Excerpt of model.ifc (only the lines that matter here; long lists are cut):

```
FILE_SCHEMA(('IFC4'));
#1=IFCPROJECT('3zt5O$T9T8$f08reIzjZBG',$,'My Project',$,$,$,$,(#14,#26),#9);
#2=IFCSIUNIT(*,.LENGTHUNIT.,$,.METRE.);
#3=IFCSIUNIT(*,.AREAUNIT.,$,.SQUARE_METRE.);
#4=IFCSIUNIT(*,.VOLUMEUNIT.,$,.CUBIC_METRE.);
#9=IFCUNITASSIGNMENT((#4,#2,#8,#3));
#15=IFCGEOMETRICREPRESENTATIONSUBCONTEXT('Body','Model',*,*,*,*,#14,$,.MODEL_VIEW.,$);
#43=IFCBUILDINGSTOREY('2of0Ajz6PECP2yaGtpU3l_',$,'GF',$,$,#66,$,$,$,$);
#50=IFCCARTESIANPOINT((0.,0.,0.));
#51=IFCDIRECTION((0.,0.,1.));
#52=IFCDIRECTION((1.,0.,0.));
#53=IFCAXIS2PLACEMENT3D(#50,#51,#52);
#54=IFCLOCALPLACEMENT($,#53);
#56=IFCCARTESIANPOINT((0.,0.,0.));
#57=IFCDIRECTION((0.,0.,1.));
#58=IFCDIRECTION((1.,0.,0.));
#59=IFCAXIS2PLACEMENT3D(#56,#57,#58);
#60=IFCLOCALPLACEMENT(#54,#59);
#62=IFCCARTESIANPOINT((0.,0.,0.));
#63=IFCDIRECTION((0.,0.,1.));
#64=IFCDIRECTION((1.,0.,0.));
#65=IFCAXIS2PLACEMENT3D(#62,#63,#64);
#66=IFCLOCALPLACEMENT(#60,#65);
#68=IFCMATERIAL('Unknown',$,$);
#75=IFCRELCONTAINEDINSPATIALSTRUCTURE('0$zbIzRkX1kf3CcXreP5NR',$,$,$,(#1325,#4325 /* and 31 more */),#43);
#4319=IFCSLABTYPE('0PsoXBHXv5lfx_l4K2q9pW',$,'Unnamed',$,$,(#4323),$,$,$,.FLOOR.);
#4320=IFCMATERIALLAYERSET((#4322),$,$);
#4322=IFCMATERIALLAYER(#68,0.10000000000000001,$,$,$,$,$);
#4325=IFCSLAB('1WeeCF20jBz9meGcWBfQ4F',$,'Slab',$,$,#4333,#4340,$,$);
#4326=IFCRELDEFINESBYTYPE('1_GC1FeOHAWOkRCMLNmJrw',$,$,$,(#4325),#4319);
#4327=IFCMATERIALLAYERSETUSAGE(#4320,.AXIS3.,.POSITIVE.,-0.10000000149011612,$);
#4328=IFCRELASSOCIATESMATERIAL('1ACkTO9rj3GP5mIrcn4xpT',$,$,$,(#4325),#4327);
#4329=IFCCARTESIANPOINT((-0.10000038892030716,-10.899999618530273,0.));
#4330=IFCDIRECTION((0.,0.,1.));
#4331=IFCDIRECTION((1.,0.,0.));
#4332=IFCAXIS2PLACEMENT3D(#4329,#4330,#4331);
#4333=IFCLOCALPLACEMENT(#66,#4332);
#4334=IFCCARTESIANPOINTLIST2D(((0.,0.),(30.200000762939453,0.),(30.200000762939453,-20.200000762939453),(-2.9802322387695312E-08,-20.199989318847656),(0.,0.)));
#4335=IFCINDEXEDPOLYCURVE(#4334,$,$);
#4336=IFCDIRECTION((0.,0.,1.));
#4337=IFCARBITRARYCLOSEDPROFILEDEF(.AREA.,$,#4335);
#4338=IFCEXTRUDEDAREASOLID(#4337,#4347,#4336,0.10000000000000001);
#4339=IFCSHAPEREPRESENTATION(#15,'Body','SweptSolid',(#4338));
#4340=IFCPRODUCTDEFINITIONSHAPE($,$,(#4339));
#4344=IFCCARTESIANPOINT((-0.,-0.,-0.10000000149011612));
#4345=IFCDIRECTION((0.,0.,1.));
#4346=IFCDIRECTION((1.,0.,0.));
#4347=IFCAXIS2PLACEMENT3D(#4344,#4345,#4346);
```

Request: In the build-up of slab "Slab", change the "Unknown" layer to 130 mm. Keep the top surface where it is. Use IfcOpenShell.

```python
import ifcopenshell
import ifcopenshell.util.element
import ifcopenshell.util.representation
import ifcopenshell.util.unit

model = ifcopenshell.open("model.ifc")
unit_scale = ifcopenshell.util.unit.calculate_unit_scale(model)

layer_set = model.by_id(4320)
layer = next(l for l in layer_set.MaterialLayers if l.Material and l.Material.Name == "Unknown")
change = 0.13 / unit_scale - layer.LayerThickness
layer.LayerThickness += change

# Geometry does not follow the layer set by itself.
slabs = [e for e in ifcopenshell.util.element.get_elements_by_material(model, layer_set) if e.is_a("IfcSlab")]
for slab in sorted(slabs, key=lambda e: e.id()):
    body = ifcopenshell.util.representation.get_representation(slab, "Model", "Body")
    solid = body.Items[0]
    old_depth = solid.Depth
    solid.Depth += change
    # Extruded upwards: lower the start of the extrusion so the top stays.
    x, y, z = solid.Position.Location.Coordinates
    solid.Position.Location = model.createIfcCartesianPoint((x, y, z - change))
    print(slab.id(), f"{old_depth:g} -> {solid.Depth:g}")

# The layers are counted up from the underside, which has moved.
for usage in {ifcopenshell.util.element.get_material(slab) for slab in slabs}:
    usage.OffsetFromReferenceLine -= change

model.write("model_edited.ifc")
```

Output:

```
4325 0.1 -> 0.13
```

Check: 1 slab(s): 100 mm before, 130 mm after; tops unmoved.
